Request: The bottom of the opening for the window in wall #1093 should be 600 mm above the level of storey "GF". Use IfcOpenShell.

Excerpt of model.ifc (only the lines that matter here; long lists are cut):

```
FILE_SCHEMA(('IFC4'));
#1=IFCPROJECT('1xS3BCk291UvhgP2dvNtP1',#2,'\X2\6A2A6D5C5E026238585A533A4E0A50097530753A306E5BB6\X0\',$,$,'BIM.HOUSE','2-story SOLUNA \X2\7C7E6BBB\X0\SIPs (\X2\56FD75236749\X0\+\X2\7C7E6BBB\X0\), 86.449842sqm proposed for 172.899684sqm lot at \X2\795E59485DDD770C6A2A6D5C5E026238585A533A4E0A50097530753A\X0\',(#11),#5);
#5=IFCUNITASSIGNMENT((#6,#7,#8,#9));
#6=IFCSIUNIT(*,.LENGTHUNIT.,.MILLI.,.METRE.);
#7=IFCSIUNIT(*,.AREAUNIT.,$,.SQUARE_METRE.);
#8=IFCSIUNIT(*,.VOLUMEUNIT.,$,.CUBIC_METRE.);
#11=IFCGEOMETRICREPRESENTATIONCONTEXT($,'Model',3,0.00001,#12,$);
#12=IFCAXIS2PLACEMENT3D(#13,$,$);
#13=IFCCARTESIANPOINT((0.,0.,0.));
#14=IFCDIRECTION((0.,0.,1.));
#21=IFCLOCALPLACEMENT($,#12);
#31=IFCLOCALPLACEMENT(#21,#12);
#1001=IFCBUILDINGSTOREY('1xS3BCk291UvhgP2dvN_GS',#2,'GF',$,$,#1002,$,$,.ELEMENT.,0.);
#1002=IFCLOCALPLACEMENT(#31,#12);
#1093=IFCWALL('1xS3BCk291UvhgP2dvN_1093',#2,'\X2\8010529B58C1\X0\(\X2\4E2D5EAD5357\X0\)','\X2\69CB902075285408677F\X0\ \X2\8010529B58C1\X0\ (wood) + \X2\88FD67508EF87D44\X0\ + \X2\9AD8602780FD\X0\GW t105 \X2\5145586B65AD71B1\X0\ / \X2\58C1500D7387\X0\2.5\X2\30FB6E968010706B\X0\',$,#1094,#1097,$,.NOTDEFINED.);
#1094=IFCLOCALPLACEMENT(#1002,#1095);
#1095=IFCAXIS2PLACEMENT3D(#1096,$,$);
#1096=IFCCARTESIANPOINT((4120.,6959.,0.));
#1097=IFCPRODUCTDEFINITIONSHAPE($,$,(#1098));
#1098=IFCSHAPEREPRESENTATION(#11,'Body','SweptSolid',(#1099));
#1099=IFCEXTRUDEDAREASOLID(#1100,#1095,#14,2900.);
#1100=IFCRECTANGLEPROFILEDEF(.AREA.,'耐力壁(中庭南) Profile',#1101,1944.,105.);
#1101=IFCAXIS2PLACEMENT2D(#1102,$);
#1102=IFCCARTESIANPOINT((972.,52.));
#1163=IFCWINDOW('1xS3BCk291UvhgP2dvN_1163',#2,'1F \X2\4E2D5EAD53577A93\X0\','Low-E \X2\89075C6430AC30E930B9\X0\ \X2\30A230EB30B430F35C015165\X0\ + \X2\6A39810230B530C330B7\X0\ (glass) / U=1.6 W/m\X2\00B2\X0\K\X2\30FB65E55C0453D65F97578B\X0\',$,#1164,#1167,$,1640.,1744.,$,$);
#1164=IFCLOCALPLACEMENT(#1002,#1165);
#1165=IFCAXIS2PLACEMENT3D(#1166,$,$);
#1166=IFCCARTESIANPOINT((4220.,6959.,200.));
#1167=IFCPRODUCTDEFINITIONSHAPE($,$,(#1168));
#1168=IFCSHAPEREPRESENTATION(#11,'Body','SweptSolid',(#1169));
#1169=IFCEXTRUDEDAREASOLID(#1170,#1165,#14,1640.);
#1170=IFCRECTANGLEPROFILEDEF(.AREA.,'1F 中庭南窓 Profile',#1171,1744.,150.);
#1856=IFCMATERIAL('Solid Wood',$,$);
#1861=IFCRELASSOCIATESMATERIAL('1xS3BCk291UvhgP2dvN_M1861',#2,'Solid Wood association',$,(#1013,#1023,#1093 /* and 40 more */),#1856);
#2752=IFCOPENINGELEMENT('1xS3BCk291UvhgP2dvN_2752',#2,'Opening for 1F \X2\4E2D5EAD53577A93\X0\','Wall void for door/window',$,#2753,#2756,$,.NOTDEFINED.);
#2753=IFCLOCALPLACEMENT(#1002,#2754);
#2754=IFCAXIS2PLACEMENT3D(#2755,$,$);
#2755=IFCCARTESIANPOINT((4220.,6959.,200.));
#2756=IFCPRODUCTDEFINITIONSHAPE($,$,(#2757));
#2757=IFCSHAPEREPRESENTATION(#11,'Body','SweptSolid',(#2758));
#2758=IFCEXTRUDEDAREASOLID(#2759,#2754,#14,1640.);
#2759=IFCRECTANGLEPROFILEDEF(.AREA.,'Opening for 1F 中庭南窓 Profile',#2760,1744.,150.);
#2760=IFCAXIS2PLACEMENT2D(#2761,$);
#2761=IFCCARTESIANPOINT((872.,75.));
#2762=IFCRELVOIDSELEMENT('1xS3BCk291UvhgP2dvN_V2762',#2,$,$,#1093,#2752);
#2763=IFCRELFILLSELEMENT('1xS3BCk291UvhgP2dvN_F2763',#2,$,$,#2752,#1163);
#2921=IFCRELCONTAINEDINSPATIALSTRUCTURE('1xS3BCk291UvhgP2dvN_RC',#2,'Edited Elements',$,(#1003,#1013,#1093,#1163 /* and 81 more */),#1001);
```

```python
import numpy as np
import ifcopenshell
import ifcopenshell.api.geometry
import ifcopenshell.geom
import ifcopenshell.util.element
import ifcopenshell.util.placement
import ifcopenshell.util.shape
import ifcopenshell.util.unit

model = ifcopenshell.open("model.ifc")
unit_scale = ifcopenshell.util.unit.calculate_unit_scale(model)

window = model.by_guid("1xS3BCk291UvhgP2dvN_1163")
opening = window.FillsVoids[0].RelatingOpeningElement
storey = ifcopenshell.util.element.get_container(window, ifc_class="IfcBuildingStorey")
level = ifcopenshell.util.placement.get_local_placement(storey.ObjectPlacement)[2, 3]

# The opening's origin need not be at the sill, so measure its lowest point.
shape = ifcopenshell.geom.create_shape(ifcopenshell.geom.settings(), opening)
bottom = ifcopenshell.util.shape.get_shape_bottom_elevation(shape, shape.geometry) / unit_scale
dz = level + 0.6 / unit_scale - bottom

shift = np.array([0.0, 0.0, dz])
# The window is not placed relative to its opening, so move both.
for product in (opening, window):
    matrix = ifcopenshell.util.placement.get_local_placement(product.ObjectPlacement)
    matrix[:3, 3] += shift
    ifcopenshell.api.geometry.edit_object_placement(model, product=product, matrix=matrix, is_si=False)

print(f"moved by {dz * unit_scale:+.3f} m")

model.write("model-out.ifc")
```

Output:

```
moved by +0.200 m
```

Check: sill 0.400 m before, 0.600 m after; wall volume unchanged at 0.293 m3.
